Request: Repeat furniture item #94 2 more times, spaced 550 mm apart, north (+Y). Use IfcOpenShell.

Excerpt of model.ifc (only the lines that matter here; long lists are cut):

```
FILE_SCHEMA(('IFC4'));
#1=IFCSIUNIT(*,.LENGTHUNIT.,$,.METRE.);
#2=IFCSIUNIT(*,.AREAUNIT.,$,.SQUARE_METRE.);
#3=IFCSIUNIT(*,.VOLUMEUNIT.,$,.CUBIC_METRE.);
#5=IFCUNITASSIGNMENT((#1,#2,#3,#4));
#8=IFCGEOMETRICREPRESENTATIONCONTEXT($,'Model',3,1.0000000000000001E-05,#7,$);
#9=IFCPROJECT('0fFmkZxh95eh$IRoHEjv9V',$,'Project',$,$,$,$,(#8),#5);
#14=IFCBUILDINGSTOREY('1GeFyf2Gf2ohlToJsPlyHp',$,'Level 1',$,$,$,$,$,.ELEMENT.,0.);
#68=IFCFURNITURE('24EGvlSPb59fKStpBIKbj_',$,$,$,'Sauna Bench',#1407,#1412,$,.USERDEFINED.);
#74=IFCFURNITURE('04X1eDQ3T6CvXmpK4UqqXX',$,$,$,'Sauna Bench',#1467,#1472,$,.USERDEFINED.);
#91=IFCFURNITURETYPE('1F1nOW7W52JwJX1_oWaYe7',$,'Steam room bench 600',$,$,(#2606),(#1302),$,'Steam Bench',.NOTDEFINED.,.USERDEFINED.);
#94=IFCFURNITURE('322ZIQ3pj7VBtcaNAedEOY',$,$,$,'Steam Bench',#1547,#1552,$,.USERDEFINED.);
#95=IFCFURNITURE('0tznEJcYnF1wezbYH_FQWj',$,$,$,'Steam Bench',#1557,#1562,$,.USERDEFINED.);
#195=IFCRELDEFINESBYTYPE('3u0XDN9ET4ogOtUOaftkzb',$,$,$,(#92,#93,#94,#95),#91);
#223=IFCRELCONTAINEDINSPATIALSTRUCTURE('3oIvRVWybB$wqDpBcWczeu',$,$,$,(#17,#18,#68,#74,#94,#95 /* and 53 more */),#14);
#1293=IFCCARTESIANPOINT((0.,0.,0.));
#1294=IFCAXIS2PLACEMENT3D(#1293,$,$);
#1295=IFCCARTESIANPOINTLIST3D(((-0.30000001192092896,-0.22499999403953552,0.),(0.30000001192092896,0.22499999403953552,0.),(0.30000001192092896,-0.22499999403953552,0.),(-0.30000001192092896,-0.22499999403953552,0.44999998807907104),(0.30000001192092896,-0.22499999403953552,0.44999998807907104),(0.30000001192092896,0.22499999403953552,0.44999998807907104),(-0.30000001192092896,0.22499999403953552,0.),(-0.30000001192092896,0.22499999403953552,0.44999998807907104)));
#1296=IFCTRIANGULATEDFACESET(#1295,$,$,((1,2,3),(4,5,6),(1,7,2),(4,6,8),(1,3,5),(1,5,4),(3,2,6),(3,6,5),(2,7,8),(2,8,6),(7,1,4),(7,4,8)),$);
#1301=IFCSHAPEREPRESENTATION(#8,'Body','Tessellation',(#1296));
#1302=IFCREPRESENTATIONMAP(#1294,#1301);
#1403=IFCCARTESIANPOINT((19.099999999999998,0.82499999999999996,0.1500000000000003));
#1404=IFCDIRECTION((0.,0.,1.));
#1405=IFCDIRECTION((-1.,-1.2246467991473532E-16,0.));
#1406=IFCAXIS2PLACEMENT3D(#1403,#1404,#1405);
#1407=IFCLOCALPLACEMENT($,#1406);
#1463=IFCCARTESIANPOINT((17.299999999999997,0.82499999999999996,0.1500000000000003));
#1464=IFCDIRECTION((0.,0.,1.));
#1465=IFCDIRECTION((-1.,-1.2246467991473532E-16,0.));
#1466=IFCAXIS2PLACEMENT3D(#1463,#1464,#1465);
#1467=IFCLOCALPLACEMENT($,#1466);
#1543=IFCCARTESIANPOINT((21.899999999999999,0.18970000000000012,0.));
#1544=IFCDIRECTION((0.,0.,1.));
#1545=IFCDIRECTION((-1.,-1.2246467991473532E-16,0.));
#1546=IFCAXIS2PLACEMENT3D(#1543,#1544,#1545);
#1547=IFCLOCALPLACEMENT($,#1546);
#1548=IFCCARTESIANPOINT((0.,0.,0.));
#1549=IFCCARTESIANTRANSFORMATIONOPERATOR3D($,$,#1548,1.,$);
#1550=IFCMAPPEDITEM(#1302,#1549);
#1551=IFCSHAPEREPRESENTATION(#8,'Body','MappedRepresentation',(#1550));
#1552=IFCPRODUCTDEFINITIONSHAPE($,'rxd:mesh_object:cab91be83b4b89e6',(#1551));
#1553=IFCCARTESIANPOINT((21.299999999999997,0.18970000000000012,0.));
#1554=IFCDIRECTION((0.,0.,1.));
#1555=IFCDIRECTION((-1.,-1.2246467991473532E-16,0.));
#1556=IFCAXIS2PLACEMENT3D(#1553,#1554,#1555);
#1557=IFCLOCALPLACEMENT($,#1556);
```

```python
import numpy as np
import ifcopenshell
import ifcopenshell.api.geometry
import ifcopenshell.api.root
import ifcopenshell.util.element
import ifcopenshell.util.placement

model = ifcopenshell.open("model.ifc")

source = model.by_guid("322ZIQ3pj7VBtcaNAedEOY")
base = ifcopenshell.util.placement.get_local_placement(source.ObjectPlacement)
step = np.array([0.0, 1.0, 0.0]) * 0.55

for i in range(1, 3):
    copy = ifcopenshell.api.root.copy_class(model, product=source)
    copy.Representation = ifcopenshell.util.element.copy_deep(
        model, source.Representation, exclude=["IfcGeometricRepresentationContext", "IfcRepresentationMap"]
    )
    matrix = base.copy()
    matrix[:3, 3] += i * step
    print("added at", matrix[:3, 3].round(3) + 0.0)
    ifcopenshell.api.geometry.edit_object_placement(model, product=copy, matrix=matrix, is_si=False)

model.write("model_edited.ifc")
```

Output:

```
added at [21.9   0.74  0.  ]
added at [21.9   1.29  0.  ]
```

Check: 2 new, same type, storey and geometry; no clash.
